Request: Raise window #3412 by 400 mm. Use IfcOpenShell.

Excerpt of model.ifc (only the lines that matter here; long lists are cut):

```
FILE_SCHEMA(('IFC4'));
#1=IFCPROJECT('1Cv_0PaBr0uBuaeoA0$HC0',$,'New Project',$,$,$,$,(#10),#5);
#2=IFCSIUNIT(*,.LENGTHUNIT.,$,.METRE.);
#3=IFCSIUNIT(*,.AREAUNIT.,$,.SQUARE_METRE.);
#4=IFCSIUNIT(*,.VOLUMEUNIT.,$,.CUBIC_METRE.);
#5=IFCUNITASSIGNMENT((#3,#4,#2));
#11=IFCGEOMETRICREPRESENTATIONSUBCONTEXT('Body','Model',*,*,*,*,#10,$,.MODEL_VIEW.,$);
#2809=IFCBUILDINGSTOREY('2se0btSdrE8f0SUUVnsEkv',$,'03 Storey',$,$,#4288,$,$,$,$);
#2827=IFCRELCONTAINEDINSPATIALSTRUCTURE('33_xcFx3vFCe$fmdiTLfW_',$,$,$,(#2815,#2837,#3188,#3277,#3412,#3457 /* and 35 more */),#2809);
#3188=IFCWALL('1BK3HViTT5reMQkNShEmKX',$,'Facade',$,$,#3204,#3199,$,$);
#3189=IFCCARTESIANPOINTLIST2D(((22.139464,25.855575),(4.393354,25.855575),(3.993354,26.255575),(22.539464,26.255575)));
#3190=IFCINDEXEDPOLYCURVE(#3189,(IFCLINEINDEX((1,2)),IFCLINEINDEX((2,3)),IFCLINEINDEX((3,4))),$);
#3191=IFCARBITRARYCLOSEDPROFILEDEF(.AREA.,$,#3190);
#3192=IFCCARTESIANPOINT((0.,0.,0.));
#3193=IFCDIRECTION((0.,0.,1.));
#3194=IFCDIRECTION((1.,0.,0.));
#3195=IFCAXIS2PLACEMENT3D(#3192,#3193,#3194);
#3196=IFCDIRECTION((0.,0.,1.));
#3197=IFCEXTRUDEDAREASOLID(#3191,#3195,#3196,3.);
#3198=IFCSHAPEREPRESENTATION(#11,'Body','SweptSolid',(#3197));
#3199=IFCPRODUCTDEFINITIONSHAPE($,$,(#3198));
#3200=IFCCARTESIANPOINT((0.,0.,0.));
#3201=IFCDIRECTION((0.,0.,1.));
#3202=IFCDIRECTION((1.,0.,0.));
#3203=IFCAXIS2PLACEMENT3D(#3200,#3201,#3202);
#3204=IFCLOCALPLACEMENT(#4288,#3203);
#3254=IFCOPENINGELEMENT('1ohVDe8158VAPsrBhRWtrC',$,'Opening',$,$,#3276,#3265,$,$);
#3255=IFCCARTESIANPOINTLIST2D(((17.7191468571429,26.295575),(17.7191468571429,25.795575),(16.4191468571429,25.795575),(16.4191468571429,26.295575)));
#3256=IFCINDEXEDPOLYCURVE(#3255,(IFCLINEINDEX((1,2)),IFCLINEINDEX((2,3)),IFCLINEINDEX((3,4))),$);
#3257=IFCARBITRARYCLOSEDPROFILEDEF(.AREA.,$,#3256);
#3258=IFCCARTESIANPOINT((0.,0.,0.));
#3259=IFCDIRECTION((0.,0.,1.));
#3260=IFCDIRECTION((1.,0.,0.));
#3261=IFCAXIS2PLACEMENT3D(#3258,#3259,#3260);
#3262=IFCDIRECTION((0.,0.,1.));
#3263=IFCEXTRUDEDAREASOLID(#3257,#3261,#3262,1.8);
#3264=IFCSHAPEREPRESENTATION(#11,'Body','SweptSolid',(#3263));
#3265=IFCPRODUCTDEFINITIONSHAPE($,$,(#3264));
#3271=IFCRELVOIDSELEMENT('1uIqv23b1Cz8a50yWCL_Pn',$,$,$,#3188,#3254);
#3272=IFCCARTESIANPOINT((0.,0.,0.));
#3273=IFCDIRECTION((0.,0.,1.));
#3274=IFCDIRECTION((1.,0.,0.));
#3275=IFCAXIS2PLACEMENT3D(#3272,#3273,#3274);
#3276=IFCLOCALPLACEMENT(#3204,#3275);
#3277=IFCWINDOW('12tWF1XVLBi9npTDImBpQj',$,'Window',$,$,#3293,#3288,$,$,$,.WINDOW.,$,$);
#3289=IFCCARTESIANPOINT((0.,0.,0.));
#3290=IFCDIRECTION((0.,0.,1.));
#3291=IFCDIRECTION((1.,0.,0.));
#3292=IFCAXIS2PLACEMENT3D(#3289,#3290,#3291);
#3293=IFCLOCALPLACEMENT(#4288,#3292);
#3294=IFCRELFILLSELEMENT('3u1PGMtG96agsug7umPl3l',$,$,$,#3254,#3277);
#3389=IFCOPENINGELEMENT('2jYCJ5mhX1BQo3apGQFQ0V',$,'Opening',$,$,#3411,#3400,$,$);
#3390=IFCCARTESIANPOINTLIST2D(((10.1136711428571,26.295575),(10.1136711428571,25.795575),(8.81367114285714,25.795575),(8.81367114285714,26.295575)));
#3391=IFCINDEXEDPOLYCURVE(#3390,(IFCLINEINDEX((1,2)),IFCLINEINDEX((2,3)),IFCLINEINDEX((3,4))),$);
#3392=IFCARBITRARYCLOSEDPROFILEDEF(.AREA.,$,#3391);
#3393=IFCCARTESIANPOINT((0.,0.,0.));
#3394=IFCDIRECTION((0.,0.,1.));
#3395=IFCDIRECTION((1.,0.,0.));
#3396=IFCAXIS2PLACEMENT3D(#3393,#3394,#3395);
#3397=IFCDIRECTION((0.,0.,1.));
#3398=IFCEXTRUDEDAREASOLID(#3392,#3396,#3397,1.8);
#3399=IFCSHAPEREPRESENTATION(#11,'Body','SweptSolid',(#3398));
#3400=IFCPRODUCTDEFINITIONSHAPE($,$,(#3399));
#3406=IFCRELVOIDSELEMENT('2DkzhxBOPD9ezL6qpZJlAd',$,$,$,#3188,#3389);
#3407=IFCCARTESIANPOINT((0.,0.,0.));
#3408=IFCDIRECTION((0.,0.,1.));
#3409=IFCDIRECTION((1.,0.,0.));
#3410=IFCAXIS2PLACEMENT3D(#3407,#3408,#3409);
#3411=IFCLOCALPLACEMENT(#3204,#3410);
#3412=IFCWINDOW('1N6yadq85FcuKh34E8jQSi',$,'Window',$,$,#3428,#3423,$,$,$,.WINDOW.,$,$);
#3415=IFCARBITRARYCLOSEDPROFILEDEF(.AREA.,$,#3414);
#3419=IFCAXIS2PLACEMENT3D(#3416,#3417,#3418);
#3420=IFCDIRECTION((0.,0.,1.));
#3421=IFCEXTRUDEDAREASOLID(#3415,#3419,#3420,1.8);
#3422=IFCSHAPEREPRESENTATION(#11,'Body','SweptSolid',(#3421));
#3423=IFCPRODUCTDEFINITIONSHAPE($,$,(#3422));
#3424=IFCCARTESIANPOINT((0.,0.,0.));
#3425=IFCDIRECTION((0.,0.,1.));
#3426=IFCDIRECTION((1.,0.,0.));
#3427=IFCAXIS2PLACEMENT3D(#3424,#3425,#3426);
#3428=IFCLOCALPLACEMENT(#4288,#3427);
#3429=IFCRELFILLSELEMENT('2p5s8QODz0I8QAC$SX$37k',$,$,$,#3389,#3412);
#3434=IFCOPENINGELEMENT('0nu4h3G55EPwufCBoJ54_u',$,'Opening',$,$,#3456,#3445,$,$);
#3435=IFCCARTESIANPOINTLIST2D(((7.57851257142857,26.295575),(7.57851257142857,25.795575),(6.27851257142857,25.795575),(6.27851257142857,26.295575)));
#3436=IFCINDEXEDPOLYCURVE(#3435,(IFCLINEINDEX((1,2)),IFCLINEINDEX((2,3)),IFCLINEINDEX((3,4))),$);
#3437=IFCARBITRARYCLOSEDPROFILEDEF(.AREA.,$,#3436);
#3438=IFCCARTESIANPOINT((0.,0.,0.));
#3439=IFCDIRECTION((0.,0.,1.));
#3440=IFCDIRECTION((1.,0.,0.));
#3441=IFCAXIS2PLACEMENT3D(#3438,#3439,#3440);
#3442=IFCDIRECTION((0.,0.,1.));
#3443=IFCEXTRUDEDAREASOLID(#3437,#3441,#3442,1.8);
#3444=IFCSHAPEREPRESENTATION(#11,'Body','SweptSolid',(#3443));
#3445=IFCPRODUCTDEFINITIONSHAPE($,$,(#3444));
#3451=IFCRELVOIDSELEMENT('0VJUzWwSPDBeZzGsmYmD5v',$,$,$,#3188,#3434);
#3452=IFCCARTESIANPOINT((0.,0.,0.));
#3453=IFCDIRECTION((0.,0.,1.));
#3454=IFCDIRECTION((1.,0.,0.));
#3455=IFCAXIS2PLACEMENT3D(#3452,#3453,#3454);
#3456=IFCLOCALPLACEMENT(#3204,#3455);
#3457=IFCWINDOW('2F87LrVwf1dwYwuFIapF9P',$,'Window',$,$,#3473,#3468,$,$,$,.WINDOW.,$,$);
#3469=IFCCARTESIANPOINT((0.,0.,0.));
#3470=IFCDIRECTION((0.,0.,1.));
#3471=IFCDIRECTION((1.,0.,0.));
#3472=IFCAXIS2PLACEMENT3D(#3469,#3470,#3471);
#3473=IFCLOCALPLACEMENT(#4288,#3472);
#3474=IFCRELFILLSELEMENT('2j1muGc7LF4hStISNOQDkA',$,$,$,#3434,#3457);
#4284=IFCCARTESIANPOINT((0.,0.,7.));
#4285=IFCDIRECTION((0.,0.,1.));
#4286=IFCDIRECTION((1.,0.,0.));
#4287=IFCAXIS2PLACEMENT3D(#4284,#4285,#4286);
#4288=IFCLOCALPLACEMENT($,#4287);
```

```python
import numpy as np
import ifcopenshell
import ifcopenshell.api.geometry
import ifcopenshell.util.placement
import ifcopenshell.util.unit

model = ifcopenshell.open("model.ifc")
unit_scale = ifcopenshell.util.unit.calculate_unit_scale(model)

window = model.by_id(3412)
opening = window.FillsVoids[0].RelatingOpeningElement
dz = 0.4 / unit_scale

shift = np.array([0.0, 0.0, dz])
# The window is not placed relative to its opening, so move both.
for product in (opening, window):
    matrix = ifcopenshell.util.placement.get_local_placement(product.ObjectPlacement)
    matrix[:3, 3] += shift
    ifcopenshell.api.geometry.edit_object_placement(model, product=product, matrix=matrix, is_si=False)

print(f"moved by {dz * unit_scale:+.3f} m")

model.write("model_updated.ifc")
```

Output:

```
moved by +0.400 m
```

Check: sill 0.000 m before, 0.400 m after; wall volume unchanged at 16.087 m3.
